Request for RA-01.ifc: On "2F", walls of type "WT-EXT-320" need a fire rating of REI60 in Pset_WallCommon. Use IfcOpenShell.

First a look at what the model holds.

```python
import ifcopenshell
import ifcopenshell.util.element

model = ifcopenshell.open("RA-01.ifc")
print(model.schema)
storey = next(s for s in model.by_type("IfcBuildingStorey") if s.Name == "2F")
walls = [e for e in ifcopenshell.util.element.get_decomposition(storey) if e.is_a("IfcWall")]
seen = {}
for e in walls:
    element_type = ifcopenshell.util.element.get_type(e)
    key = (element_type.Name if element_type != e and element_type else None, ifcopenshell.util.element.get_pset(e, "Pset_WallCommon", "FireRating"))
    seen[key] = seen.get(key, 0) + 1
for (name, value), count in sorted(seen.items(), key=str):
    print(count, "x", name, "|", value)
```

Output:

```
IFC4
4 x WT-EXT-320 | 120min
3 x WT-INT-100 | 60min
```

```python
import ifcopenshell
import ifcopenshell.api.pset
import ifcopenshell.util.element

model = ifcopenshell.open("RA-01.ifc")

storey = next(s for s in model.by_type("IfcBuildingStorey") if s.Name == "2F")
walls = [e for e in ifcopenshell.util.element.get_decomposition(storey) if e.is_a("IfcWall")]

count = 0
for e in walls:
    element_type = ifcopenshell.util.element.get_type(e)
    if element_type in (None, e) or element_type.Name != "WT-EXT-320":
        continue
    # add_pset returns the element's existing set when there is one.
    pset = ifcopenshell.api.pset.add_pset(model, product=e, name="Pset_WallCommon")
    ifcopenshell.api.pset.edit_pset(model, pset=pset, properties={"FireRating": "REI60"})
    count += 1

print(count, "walls updated")

model.write("RA-01_updated.ifc")
```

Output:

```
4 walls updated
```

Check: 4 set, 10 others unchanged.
